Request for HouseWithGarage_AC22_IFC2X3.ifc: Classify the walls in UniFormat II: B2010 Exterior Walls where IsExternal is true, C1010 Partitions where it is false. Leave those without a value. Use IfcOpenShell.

First a look at what the model holds.

```python
import ifcopenshell
import ifcopenshell.util.element

model = ifcopenshell.open("HouseWithGarage_AC22_IFC2X3.ifc")
print(model.schema)
print("classifications:", [c.Name for c in model.by_type("IfcClassification")])
values = [ifcopenshell.util.element.get_pset(e, "Pset_WallCommon", "IsExternal") for e in model.by_type("IfcWall")]
for value in (True, False, None):
    print("IsExternal", value, values.count(value))
```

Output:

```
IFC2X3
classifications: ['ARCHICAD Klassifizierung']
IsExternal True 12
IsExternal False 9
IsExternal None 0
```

```python
import ifcopenshell
import ifcopenshell.api.classification
import ifcopenshell.util.element

model = ifcopenshell.open("HouseWithGarage_AC22_IFC2X3.ifc")

# IFC2X3 requires Source and Edition and has no link from the project to the system.
system = model.create_entity("IfcClassification", Source="ASTM", Edition="E1557", Name="UniFormat II")

walls = model.by_type("IfcWall")
external = {e: ifcopenshell.util.element.get_pset(e, "Pset_WallCommon", "IsExternal") for e in walls}
for flag, code, name in ((True, "B2010", "Exterior Walls"), (False, "C1010", "Partitions")):
    products = [e for e in walls if external[e] is flag]
    ifcopenshell.api.classification.add_reference(
        model, products=products, classification=system, identification=code, name=name
    )
    print(code, len(products))

model.write("HouseWithGarage_AC22_IFC2X3-out.ifc")
```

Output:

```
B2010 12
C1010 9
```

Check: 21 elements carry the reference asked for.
